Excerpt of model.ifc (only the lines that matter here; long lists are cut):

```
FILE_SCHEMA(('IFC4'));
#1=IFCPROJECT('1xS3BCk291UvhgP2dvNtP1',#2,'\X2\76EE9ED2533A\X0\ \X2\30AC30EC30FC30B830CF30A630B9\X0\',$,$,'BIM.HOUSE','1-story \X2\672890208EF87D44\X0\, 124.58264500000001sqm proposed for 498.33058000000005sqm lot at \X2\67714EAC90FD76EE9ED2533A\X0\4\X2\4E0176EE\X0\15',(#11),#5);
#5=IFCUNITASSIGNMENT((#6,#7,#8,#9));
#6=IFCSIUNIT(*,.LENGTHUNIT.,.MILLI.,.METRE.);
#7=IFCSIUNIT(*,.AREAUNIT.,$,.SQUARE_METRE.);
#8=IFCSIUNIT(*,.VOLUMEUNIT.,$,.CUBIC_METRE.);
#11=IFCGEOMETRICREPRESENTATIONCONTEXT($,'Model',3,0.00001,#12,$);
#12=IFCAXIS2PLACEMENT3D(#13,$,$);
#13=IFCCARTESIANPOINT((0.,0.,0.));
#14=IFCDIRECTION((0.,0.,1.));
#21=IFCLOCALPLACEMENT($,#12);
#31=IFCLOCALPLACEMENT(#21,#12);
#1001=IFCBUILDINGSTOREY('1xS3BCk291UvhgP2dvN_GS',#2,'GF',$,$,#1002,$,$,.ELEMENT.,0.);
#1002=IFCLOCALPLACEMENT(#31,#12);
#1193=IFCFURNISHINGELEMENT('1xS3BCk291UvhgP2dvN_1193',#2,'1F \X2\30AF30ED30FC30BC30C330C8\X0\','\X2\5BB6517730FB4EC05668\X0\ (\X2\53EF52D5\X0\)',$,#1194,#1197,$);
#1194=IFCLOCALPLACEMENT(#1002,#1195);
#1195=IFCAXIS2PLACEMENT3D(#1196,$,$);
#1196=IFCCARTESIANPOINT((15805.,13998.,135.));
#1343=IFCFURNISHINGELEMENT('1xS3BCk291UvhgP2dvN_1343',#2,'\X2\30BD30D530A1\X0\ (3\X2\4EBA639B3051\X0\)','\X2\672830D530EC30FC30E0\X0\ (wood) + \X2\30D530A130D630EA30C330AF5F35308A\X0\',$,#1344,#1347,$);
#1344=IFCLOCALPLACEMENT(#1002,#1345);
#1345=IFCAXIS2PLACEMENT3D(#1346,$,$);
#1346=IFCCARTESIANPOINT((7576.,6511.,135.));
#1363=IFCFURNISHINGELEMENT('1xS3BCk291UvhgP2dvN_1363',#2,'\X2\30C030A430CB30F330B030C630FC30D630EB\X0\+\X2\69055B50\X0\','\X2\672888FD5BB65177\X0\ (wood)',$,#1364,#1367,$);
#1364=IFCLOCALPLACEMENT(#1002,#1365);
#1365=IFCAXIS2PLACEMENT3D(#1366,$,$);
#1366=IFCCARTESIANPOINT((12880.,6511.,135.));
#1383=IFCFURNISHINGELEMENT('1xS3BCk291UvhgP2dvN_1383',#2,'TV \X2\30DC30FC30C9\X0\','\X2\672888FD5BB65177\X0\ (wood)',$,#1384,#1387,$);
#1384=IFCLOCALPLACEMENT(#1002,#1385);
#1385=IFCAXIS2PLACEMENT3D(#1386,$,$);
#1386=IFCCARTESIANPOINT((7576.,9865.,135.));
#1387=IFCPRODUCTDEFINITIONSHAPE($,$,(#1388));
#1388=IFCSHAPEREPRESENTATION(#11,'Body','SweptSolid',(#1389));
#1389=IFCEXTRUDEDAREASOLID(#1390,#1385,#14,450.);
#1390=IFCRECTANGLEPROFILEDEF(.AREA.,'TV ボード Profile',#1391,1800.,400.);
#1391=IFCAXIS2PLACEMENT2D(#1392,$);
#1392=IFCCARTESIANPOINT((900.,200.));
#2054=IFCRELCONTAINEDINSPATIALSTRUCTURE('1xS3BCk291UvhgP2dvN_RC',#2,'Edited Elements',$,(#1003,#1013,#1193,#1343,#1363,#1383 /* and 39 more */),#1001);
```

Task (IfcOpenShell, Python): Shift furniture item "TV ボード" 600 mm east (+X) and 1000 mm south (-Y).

```python
import ifcopenshell
import ifcopenshell.api.geometry
import ifcopenshell.util.placement
import ifcopenshell.util.unit

model = ifcopenshell.open("model.ifc")
unit_scale = ifcopenshell.util.unit.calculate_unit_scale(model)

item = model.by_id(1383)
matrix = ifcopenshell.util.placement.get_local_placement(item.ObjectPlacement)
matrix[0, 3] += 0.6 / unit_scale
matrix[1, 3] -= 1 / unit_scale
ifcopenshell.api.geometry.edit_object_placement(model, product=item, matrix=matrix, is_si=False)

print(ifcopenshell.util.placement.get_local_placement(item.ObjectPlacement).round(3) + 0.0)

model.write("model_updated.ifc")
```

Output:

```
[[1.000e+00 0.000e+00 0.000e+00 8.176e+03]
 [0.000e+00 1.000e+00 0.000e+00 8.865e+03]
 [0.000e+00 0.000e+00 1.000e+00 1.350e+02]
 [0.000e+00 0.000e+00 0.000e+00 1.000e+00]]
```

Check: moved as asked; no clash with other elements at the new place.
